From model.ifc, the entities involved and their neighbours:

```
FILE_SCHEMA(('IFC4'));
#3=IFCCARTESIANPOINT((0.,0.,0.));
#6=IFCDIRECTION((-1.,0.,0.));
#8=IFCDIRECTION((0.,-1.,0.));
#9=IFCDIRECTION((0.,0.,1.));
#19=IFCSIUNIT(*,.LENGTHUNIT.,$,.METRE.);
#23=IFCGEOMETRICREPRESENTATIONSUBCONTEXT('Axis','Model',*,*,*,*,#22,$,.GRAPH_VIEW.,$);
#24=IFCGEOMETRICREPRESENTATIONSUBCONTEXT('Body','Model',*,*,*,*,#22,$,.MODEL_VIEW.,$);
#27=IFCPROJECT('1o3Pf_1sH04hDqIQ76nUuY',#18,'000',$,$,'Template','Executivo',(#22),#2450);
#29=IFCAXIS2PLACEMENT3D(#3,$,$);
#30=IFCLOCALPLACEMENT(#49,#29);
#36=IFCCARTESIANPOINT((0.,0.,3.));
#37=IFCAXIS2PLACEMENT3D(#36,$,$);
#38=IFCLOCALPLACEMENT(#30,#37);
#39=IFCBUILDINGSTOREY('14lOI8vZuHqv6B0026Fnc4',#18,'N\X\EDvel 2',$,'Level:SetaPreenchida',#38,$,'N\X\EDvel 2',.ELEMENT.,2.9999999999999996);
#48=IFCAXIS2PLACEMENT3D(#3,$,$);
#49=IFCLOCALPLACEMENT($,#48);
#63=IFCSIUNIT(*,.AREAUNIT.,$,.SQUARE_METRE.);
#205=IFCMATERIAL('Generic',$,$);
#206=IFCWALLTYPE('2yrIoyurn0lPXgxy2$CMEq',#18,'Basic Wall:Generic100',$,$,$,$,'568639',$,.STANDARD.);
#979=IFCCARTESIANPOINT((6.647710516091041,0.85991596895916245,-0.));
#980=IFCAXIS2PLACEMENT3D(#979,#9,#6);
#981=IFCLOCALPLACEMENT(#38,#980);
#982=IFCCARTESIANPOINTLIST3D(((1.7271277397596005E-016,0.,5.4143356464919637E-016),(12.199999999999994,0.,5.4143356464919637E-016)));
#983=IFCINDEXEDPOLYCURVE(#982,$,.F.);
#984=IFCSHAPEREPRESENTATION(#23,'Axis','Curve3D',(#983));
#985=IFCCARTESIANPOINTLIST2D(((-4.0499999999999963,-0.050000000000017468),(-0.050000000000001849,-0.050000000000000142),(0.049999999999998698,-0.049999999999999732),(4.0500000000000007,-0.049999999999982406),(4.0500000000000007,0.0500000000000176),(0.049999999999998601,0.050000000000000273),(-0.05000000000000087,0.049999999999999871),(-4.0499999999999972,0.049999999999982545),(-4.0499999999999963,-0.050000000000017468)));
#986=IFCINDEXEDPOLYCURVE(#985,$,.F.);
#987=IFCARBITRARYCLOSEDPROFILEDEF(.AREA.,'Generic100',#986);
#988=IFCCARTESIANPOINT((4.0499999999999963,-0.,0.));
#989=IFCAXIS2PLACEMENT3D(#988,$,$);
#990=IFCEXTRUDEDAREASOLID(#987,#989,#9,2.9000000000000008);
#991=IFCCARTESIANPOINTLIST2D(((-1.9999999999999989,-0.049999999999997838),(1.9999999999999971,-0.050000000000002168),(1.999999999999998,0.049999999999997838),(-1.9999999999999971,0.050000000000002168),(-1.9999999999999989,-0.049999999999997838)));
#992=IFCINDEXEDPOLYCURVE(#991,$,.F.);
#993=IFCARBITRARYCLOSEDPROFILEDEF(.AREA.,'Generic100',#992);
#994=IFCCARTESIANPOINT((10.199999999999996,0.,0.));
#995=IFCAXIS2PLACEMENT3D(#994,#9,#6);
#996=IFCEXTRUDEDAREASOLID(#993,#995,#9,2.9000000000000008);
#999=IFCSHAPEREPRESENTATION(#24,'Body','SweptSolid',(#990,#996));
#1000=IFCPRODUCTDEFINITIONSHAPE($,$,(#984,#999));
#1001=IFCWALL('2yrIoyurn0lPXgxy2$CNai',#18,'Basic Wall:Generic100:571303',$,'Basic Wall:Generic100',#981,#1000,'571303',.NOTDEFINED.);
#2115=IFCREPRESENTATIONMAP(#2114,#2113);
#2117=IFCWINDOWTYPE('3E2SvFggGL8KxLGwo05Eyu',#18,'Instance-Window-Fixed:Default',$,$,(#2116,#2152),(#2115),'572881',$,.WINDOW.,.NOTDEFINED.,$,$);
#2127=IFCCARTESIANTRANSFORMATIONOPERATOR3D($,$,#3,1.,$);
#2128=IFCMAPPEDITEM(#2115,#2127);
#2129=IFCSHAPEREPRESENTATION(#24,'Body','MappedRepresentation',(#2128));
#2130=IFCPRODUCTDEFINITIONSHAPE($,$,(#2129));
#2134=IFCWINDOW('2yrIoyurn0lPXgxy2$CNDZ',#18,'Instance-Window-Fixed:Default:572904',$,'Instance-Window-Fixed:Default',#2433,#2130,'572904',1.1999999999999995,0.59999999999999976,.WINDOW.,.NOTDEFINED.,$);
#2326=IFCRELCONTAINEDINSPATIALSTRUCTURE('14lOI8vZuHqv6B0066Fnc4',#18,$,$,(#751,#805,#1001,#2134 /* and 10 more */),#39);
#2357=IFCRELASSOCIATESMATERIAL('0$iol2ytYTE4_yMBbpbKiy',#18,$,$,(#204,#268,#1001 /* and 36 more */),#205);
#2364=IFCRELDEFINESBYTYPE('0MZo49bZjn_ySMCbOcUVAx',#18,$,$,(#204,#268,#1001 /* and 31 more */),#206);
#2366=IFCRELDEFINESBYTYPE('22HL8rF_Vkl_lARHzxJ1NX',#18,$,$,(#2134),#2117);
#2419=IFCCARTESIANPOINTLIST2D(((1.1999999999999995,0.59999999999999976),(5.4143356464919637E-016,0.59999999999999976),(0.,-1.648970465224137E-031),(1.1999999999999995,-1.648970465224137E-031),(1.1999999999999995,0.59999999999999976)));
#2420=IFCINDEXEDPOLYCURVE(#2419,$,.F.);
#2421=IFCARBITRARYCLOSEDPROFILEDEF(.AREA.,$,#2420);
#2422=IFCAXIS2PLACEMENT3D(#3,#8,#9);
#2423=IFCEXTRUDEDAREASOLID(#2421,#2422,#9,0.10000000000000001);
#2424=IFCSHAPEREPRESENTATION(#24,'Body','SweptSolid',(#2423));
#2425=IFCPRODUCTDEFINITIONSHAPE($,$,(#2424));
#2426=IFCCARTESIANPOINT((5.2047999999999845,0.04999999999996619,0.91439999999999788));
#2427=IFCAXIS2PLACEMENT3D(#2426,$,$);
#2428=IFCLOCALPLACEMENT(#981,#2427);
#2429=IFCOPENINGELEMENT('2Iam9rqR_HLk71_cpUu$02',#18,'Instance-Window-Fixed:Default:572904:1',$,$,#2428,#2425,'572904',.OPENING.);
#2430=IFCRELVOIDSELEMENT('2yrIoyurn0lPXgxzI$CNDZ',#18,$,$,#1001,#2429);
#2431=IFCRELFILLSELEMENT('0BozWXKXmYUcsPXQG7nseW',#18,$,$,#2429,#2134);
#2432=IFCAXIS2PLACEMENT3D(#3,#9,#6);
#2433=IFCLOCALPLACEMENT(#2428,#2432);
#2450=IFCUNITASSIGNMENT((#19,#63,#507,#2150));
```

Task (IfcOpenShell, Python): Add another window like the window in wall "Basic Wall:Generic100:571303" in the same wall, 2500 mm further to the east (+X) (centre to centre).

```python
import ifcopenshell
import ifcopenshell.api.feature
import ifcopenshell.api.geometry
import ifcopenshell.api.root
import ifcopenshell.geom
import ifcopenshell.util.element
import ifcopenshell.util.placement
import ifcopenshell.util.shape
import ifcopenshell.util.unit

model = ifcopenshell.open("model.ifc")
unit_scale = ifcopenshell.util.unit.calculate_unit_scale(model)
settings = ifcopenshell.geom.settings()


def volume(element):
    """Net volume in cubic metres, openings subtracted."""
    shape = ifcopenshell.geom.create_shape(settings, element)
    return ifcopenshell.util.shape.get_volume(shape.geometry)


def reuse_history(source, copy):
    """copy_class also copies each property set's owner history, people and application; keep the originals."""
    for rel in copy.IsDefinedBy:
        if rel.is_a("IfcRelDefinesByProperties") and (history := rel.RelatingPropertyDefinition.OwnerHistory):
            rel.RelatingPropertyDefinition.OwnerHistory = source.OwnerHistory
            ifcopenshell.util.element.remove_deep2(model, history)


window = model.by_id(2134)
opening = window.FillsVoids[0].RelatingOpeningElement
wall = opening.VoidsElements[0].RelatingBuildingElement
before = volume(wall)
shift = ifcopenshell.util.placement.get_local_placement(wall.ObjectPlacement)[:3, 0] * -2.5 / unit_scale

# copy_class copies the void relationship, type, container and properties, but no geometry.
new_opening = ifcopenshell.api.root.copy_class(model, product=opening)
new_opening.Representation = ifcopenshell.util.element.copy_deep(
    model, opening.Representation, exclude=["IfcGeometricRepresentationContext", "IfcRepresentationMap"]
)
new_opening.Name = "Instance-Window-Fixed:Default"
new_opening.Tag = None
new_window = ifcopenshell.api.root.copy_class(model, product=window)
new_window.Representation = ifcopenshell.util.element.copy_deep(
    model, window.Representation, exclude=["IfcGeometricRepresentationContext", "IfcRepresentationMap"]
)
new_window.Name = "Instance-Window-Fixed:Default"
new_window.Tag = None
reuse_history(window, new_window)
ifcopenshell.api.feature.add_filling(model, opening=new_opening, element=new_window)

for old, new in ((opening, new_opening), (window, new_window)):
    matrix = ifcopenshell.util.placement.get_local_placement(old.ObjectPlacement)
    matrix[:3, 3] += shift
    ifcopenshell.api.geometry.edit_object_placement(model, product=new, matrix=matrix, is_si=False)

after = volume(wall)

print(f"wall volume {before:.3f} -> {after:.3f} m3")

model.write("model-out.ifc")
```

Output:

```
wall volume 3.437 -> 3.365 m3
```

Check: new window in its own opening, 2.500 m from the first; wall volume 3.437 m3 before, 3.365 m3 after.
